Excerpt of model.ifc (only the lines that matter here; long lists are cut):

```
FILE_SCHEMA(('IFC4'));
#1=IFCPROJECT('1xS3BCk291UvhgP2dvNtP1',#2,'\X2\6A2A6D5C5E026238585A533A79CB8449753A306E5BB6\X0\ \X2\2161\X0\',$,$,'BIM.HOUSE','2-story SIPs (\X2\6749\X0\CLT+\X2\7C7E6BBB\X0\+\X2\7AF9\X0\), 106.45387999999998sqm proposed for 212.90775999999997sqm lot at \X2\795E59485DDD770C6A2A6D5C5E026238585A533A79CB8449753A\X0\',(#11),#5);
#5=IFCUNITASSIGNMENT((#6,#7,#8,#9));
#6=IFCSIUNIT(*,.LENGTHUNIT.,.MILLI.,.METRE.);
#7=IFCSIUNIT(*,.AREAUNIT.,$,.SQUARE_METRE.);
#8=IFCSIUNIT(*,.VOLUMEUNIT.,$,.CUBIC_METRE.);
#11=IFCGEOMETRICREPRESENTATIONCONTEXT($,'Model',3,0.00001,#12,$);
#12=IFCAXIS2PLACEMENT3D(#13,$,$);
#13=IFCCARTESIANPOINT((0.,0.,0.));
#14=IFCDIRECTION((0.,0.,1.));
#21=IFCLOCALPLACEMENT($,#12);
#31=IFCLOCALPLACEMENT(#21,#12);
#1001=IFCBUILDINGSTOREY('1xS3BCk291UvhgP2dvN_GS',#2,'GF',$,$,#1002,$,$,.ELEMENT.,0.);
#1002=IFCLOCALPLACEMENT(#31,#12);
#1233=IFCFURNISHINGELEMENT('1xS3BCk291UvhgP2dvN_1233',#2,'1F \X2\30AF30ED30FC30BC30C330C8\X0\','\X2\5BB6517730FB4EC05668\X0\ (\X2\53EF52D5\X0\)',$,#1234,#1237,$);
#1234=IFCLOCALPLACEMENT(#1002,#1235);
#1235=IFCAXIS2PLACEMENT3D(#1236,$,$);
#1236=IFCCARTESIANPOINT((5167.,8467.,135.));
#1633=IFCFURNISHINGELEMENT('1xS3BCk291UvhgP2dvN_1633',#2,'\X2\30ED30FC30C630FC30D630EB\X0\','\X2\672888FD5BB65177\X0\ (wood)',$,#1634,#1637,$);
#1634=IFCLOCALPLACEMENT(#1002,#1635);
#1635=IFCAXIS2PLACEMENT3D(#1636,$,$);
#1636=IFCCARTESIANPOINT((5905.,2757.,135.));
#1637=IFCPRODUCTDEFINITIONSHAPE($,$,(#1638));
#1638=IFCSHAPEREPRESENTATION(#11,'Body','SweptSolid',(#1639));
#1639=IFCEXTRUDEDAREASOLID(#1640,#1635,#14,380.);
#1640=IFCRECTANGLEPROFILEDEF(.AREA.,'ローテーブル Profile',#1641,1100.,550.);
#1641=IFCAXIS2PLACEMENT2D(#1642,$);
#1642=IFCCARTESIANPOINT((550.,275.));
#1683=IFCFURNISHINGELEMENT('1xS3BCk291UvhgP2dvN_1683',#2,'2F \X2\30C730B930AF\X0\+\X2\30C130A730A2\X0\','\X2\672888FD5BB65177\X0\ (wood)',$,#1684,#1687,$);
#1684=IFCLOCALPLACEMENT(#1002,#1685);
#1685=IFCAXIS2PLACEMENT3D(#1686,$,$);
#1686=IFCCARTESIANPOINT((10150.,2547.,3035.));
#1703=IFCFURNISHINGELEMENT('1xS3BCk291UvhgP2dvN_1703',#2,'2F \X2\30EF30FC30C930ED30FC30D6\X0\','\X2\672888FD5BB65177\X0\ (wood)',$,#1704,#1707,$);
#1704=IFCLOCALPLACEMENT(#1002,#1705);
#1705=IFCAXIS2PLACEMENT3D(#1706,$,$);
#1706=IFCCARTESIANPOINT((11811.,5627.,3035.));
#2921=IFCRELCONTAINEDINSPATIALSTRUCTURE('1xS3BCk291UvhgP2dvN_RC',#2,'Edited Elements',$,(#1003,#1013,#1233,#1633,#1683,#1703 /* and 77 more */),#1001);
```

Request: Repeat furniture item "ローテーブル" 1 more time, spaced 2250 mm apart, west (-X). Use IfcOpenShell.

```python
import numpy as np
import ifcopenshell
import ifcopenshell.api.geometry
import ifcopenshell.api.root
import ifcopenshell.util.element
import ifcopenshell.util.placement
import ifcopenshell.util.unit

model = ifcopenshell.open("model.ifc")
unit_scale = ifcopenshell.util.unit.calculate_unit_scale(model)


def reuse_history(source, copy):
    """copy_class also copies each property set's owner history, people and application; keep the originals."""
    for rel in copy.IsDefinedBy:
        if rel.is_a("IfcRelDefinesByProperties") and (history := rel.RelatingPropertyDefinition.OwnerHistory):
            rel.RelatingPropertyDefinition.OwnerHistory = source.OwnerHistory
            ifcopenshell.util.element.remove_deep2(model, history)


source = model.by_id(1633)
base = ifcopenshell.util.placement.get_local_placement(source.ObjectPlacement)
step = np.array([-1.0, 0.0, 0.0]) * 2.25 / unit_scale

for i in range(1, 2):
    copy = ifcopenshell.api.root.copy_class(model, product=source)
    copy.Representation = ifcopenshell.util.element.copy_deep(
        model, source.Representation, exclude=["IfcGeometricRepresentationContext", "IfcRepresentationMap"]
    )
    reuse_history(source, copy)
    matrix = base.copy()
    matrix[:3, 3] += i * step
    print("added at", matrix[:3, 3].round(3) + 0.0)
    ifcopenshell.api.geometry.edit_object_placement(model, product=copy, matrix=matrix, is_si=False)

model.write("model_v2.ifc")
```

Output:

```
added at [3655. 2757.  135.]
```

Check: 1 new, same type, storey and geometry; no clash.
